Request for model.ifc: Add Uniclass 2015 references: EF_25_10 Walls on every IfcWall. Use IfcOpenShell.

First a look at what the model holds.

```python
import ifcopenshell

model = ifcopenshell.open("model.ifc")
print(model.schema)
print("classifications:", [c.Name for c in model.by_type("IfcClassification")])
for ifc_class in ("IfcDoor", "IfcRoof", "IfcStair", "IfcWall", "IfcWindow"):
    print(ifc_class, len(model.by_type(ifc_class)))
```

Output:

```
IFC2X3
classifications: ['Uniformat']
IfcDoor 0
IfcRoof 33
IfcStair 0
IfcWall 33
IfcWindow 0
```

```python
import ifcopenshell
import ifcopenshell.api.classification

model = ifcopenshell.open("model.ifc")

# IFC2X3 requires Source and Edition and has no link from the project to the system.
system = model.create_entity("IfcClassification", Source="NBS", Edition="2015", Name="Uniclass 2015")

codes = {
    "IfcWall": ("EF_25_10", "Walls"),
}
for ifc_class, (code, name) in codes.items():
    products = model.by_type(ifc_class)
    ifcopenshell.api.classification.add_reference(
        model, products=products, classification=system, identification=code, name=name
    )
    print(code, len(products))

model.write("model_rev.ifc")
```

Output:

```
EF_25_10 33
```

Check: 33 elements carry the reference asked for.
